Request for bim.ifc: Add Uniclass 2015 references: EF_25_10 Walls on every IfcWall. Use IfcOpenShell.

First a look at what the model holds.

```python
import ifcopenshell

model = ifcopenshell.open("bim.ifc")
print(model.schema)
print("classifications:", [c.Name for c in model.by_type("IfcClassification")])
for ifc_class in ("IfcDoor", "IfcRoof", "IfcStair", "IfcWall", "IfcWindow"):
    print(ifc_class, len(model.by_type(ifc_class)))
```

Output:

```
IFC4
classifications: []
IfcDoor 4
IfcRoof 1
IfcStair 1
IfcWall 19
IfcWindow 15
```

```python
import ifcopenshell
import ifcopenshell.api.classification

model = ifcopenshell.open("bim.ifc")

system = ifcopenshell.api.classification.add_classification(model, classification="Uniclass 2015")

codes = {
    "IfcWall": ("EF_25_10", "Walls"),
}
for ifc_class, (code, name) in codes.items():
    products = model.by_type(ifc_class)
    ifcopenshell.api.classification.add_reference(
        model, products=products, classification=system, identification=code, name=name
    )
    print(code, len(products))

model.write("bim_edited.ifc")
```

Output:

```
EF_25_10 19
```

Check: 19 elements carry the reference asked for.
